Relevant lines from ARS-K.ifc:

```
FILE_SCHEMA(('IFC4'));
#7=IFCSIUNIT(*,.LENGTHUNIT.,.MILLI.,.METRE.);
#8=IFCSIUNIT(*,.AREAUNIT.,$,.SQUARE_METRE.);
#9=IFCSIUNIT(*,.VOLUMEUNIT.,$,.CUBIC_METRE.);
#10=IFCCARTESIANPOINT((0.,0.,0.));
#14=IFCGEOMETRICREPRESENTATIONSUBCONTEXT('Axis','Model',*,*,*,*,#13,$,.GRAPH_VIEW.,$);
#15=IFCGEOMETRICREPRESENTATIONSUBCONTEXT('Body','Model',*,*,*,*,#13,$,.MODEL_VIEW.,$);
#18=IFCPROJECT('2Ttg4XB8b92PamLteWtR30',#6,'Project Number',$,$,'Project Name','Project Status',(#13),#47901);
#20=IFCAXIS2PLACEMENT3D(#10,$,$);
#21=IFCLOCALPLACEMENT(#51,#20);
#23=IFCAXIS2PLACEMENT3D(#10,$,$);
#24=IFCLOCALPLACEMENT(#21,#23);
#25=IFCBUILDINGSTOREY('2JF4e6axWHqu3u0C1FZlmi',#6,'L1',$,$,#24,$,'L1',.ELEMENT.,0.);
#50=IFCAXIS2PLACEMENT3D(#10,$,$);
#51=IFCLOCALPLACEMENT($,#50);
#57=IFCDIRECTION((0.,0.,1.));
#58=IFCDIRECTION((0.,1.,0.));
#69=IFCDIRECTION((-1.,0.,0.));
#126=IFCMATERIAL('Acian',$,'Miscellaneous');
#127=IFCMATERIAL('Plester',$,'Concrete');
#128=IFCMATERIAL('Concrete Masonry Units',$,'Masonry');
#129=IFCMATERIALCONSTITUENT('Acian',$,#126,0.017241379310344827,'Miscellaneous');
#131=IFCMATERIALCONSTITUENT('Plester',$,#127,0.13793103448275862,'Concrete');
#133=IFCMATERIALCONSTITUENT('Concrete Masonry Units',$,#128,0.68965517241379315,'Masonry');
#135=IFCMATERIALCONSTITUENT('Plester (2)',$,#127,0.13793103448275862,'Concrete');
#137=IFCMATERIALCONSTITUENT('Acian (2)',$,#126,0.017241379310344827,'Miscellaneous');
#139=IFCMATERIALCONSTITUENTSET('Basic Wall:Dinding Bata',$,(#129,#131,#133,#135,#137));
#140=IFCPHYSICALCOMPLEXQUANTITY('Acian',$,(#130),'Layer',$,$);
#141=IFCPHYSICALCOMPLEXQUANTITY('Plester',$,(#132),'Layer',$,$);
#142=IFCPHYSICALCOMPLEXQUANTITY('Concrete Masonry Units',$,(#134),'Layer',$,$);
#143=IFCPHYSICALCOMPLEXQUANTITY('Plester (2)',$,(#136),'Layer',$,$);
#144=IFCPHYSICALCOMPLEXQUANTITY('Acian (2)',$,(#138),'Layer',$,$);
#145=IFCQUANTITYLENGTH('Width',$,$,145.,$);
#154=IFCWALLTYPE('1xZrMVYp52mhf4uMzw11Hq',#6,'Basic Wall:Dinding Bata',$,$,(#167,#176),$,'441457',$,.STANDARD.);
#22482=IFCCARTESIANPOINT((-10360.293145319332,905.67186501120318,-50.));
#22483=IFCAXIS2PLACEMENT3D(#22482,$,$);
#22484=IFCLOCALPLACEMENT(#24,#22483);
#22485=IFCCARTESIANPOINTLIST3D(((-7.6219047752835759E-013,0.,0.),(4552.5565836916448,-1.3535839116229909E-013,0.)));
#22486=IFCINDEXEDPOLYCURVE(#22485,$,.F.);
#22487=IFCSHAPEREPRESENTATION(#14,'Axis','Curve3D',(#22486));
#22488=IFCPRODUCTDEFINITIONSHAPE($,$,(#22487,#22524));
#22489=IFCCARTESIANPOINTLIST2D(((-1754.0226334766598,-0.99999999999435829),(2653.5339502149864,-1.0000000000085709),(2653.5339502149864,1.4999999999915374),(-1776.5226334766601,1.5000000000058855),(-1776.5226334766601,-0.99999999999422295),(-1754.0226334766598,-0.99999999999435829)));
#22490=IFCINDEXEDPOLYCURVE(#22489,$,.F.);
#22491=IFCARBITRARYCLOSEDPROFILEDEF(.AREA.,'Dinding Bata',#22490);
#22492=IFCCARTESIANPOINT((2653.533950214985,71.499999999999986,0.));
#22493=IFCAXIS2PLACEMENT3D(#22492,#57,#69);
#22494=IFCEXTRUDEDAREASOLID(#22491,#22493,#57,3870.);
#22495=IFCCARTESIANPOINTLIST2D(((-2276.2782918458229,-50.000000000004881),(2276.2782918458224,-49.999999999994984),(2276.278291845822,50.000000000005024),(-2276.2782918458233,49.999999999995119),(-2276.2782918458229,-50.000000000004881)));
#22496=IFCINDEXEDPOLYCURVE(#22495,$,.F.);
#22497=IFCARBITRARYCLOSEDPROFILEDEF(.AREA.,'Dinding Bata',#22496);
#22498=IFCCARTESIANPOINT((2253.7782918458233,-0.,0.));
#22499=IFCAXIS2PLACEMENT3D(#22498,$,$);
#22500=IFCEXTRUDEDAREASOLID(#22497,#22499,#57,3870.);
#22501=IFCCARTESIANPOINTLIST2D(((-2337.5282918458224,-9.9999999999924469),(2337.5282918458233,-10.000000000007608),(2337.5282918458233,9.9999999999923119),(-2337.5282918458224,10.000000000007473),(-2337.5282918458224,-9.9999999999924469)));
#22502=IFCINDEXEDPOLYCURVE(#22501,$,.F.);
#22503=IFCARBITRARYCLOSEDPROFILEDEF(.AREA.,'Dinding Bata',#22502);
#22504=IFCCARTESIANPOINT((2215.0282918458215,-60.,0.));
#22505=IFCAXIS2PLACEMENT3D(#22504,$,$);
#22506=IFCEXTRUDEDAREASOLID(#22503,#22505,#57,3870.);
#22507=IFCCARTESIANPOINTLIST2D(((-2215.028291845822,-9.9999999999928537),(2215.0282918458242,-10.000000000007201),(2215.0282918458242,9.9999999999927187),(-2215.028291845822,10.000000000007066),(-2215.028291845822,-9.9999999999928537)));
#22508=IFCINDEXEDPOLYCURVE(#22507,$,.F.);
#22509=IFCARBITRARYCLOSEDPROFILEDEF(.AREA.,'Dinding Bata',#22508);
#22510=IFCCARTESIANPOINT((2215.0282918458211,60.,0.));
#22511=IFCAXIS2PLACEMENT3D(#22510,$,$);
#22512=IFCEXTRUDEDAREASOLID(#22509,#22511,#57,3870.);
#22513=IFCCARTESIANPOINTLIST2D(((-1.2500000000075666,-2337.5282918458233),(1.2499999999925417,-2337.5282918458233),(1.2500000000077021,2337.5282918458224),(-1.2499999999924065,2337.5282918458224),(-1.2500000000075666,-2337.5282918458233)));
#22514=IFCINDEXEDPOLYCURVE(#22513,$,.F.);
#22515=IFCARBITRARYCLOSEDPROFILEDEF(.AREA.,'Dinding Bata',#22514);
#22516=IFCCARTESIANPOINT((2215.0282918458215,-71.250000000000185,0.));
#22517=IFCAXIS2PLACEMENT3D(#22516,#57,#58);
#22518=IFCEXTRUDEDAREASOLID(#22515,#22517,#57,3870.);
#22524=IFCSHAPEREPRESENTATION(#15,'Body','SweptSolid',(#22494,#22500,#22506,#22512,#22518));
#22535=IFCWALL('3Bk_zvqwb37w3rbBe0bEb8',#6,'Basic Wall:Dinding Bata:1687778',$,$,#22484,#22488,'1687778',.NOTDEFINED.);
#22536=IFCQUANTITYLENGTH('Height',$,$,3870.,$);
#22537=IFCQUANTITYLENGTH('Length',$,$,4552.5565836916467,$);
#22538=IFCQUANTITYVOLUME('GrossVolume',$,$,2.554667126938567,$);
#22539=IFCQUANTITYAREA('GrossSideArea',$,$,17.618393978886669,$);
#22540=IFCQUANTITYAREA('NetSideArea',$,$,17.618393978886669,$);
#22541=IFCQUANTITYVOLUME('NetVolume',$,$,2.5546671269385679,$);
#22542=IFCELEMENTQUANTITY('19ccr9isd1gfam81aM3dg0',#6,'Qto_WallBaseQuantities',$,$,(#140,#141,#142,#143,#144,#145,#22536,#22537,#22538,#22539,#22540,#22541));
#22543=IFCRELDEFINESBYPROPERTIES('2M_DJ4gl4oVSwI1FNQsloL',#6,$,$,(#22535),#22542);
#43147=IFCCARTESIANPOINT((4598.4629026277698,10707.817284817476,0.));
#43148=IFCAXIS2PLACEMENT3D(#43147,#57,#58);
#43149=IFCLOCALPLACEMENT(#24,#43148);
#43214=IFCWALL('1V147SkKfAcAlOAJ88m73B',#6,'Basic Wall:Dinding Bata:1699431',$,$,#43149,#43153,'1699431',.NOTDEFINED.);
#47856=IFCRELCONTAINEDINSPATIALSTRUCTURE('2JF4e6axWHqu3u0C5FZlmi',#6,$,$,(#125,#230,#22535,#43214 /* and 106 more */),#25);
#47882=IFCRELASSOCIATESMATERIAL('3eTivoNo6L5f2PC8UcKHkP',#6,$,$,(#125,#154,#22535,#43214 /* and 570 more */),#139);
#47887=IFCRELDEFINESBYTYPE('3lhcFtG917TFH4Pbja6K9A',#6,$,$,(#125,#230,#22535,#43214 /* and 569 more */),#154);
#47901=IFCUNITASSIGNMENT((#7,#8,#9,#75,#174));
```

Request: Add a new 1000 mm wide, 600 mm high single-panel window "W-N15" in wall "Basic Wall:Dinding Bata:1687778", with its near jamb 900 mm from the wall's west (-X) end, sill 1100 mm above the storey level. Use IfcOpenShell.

```python
import numpy as np
import ifcopenshell
import ifcopenshell.api.feature
import ifcopenshell.api.geometry
import ifcopenshell.api.pset
import ifcopenshell.api.root
import ifcopenshell.api.spatial
import ifcopenshell.geom
import ifcopenshell.util.element
import ifcopenshell.util.placement
import ifcopenshell.util.representation
import ifcopenshell.util.shape
import ifcopenshell.util.unit

model = ifcopenshell.open("ARS-K.ifc")
unit_scale = ifcopenshell.util.unit.calculate_unit_scale(model)
area_scale = ifcopenshell.util.unit.calculate_unit_scale(model, "AREAUNIT")
volume_scale = ifcopenshell.util.unit.calculate_unit_scale(model, "VOLUMEUNIT")
settings = ifcopenshell.geom.settings()


def volume(element):
    """Net volume in cubic metres, openings subtracted."""
    shape = ifcopenshell.geom.create_shape(settings, element)
    return ifcopenshell.util.shape.get_volume(shape.geometry)


wall = model.by_id(22535)
storey = ifcopenshell.util.element.get_container(wall, ifc_class="IfcBuildingStorey")
context = ifcopenshell.util.representation.get_context(model, "Model", "Body", "MODEL_VIEW")
before = volume(wall)

width, height, from_end, sill = 1, 0.6, 0.9, 1.1  # metres

# The wall runs along its own X axis, and the end named is its -X end.
wall_shape = ifcopenshell.geom.create_shape(settings, wall)
x, y, z = ifcopenshell.util.shape.get_vertices(wall_shape.geometry).T
start = x.min() + from_end
face, thickness = float(y.min()), float(y.max() - y.min())
wall_matrix = ifcopenshell.util.placement.get_local_placement(wall.ObjectPlacement)
level = ifcopenshell.util.placement.get_local_placement(storey.ObjectPlacement)[2, 3]


def in_wall(x, y):
    """Placement at x, y metres in the wall's axes, at sill height."""
    matrix = wall_matrix.copy()
    matrix[:, 3] = wall_matrix @ np.array([x / unit_scale, y / unit_scale, 0.0, 1.0])
    matrix[2, 3] = level + sill / unit_scale
    return matrix


# Opening: a box that overshoots both wall faces by 50 mm.
opening = ifcopenshell.api.root.create_entity(model, ifc_class="IfcOpeningElement", predefined_type="OPENING")
box = ifcopenshell.api.geometry.add_wall_representation(
    model, context=context, length=width, height=height, thickness=thickness + 0.1
)
ifcopenshell.api.geometry.assign_representation(model, product=opening, representation=box)
ifcopenshell.api.geometry.edit_object_placement(model, product=opening, matrix=in_wall(start, face - 0.05), is_si=False)
ifcopenshell.api.feature.add_feature(model, feature=opening, element=wall)

window = ifcopenshell.api.root.create_entity(model, ifc_class="IfcWindow", name="W-N15", predefined_type="WINDOW")
window.OverallWidth, window.OverallHeight = width / unit_scale, height / unit_scale
window.PartitioningType = "SINGLE_PANEL"
body = ifcopenshell.api.geometry.add_window_representation(
    model,
    context=context,
    overall_width=window.OverallWidth,
    overall_height=window.OverallHeight,
    partition_type="SINGLE_PANEL",
)
ifcopenshell.api.geometry.assign_representation(model, product=window, representation=body)
ifcopenshell.api.spatial.assign_container(model, products=[window], relating_structure=storey)
ifcopenshell.api.feature.add_filling(model, opening=opening, element=window)

# Centre the window in the wall's thickness.
ifcopenshell.api.geometry.edit_object_placement(model, product=window, matrix=in_wall(start, face), is_si=False)
window_shape = ifcopenshell.geom.create_shape(settings, window)
depth = ifcopenshell.util.shape.get_vertices(window_shape.geometry)[:, 1]
offset = face + thickness / 2 - (depth.min() + depth.max()) / 2
ifcopenshell.api.geometry.edit_object_placement(model, product=window, matrix=in_wall(start, offset), is_si=False)

after = volume(wall)

# Update the wall's stored quantities.
qto = model.by_id(ifcopenshell.util.element.get_pset(wall, "Qto_WallBaseQuantities", should_inherit=False)["id"])
ifcopenshell.api.pset.edit_qto(model, qto=qto, properties={
    "NetSideArea": after / thickness / area_scale,
    "NetVolume": after / volume_scale,
})

print(f"wall volume {before:.3f} -> {after:.3f} m3")

model.write("ARS-K_edited.ifc")
```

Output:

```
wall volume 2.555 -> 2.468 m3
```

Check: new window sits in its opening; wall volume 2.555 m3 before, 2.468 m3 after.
